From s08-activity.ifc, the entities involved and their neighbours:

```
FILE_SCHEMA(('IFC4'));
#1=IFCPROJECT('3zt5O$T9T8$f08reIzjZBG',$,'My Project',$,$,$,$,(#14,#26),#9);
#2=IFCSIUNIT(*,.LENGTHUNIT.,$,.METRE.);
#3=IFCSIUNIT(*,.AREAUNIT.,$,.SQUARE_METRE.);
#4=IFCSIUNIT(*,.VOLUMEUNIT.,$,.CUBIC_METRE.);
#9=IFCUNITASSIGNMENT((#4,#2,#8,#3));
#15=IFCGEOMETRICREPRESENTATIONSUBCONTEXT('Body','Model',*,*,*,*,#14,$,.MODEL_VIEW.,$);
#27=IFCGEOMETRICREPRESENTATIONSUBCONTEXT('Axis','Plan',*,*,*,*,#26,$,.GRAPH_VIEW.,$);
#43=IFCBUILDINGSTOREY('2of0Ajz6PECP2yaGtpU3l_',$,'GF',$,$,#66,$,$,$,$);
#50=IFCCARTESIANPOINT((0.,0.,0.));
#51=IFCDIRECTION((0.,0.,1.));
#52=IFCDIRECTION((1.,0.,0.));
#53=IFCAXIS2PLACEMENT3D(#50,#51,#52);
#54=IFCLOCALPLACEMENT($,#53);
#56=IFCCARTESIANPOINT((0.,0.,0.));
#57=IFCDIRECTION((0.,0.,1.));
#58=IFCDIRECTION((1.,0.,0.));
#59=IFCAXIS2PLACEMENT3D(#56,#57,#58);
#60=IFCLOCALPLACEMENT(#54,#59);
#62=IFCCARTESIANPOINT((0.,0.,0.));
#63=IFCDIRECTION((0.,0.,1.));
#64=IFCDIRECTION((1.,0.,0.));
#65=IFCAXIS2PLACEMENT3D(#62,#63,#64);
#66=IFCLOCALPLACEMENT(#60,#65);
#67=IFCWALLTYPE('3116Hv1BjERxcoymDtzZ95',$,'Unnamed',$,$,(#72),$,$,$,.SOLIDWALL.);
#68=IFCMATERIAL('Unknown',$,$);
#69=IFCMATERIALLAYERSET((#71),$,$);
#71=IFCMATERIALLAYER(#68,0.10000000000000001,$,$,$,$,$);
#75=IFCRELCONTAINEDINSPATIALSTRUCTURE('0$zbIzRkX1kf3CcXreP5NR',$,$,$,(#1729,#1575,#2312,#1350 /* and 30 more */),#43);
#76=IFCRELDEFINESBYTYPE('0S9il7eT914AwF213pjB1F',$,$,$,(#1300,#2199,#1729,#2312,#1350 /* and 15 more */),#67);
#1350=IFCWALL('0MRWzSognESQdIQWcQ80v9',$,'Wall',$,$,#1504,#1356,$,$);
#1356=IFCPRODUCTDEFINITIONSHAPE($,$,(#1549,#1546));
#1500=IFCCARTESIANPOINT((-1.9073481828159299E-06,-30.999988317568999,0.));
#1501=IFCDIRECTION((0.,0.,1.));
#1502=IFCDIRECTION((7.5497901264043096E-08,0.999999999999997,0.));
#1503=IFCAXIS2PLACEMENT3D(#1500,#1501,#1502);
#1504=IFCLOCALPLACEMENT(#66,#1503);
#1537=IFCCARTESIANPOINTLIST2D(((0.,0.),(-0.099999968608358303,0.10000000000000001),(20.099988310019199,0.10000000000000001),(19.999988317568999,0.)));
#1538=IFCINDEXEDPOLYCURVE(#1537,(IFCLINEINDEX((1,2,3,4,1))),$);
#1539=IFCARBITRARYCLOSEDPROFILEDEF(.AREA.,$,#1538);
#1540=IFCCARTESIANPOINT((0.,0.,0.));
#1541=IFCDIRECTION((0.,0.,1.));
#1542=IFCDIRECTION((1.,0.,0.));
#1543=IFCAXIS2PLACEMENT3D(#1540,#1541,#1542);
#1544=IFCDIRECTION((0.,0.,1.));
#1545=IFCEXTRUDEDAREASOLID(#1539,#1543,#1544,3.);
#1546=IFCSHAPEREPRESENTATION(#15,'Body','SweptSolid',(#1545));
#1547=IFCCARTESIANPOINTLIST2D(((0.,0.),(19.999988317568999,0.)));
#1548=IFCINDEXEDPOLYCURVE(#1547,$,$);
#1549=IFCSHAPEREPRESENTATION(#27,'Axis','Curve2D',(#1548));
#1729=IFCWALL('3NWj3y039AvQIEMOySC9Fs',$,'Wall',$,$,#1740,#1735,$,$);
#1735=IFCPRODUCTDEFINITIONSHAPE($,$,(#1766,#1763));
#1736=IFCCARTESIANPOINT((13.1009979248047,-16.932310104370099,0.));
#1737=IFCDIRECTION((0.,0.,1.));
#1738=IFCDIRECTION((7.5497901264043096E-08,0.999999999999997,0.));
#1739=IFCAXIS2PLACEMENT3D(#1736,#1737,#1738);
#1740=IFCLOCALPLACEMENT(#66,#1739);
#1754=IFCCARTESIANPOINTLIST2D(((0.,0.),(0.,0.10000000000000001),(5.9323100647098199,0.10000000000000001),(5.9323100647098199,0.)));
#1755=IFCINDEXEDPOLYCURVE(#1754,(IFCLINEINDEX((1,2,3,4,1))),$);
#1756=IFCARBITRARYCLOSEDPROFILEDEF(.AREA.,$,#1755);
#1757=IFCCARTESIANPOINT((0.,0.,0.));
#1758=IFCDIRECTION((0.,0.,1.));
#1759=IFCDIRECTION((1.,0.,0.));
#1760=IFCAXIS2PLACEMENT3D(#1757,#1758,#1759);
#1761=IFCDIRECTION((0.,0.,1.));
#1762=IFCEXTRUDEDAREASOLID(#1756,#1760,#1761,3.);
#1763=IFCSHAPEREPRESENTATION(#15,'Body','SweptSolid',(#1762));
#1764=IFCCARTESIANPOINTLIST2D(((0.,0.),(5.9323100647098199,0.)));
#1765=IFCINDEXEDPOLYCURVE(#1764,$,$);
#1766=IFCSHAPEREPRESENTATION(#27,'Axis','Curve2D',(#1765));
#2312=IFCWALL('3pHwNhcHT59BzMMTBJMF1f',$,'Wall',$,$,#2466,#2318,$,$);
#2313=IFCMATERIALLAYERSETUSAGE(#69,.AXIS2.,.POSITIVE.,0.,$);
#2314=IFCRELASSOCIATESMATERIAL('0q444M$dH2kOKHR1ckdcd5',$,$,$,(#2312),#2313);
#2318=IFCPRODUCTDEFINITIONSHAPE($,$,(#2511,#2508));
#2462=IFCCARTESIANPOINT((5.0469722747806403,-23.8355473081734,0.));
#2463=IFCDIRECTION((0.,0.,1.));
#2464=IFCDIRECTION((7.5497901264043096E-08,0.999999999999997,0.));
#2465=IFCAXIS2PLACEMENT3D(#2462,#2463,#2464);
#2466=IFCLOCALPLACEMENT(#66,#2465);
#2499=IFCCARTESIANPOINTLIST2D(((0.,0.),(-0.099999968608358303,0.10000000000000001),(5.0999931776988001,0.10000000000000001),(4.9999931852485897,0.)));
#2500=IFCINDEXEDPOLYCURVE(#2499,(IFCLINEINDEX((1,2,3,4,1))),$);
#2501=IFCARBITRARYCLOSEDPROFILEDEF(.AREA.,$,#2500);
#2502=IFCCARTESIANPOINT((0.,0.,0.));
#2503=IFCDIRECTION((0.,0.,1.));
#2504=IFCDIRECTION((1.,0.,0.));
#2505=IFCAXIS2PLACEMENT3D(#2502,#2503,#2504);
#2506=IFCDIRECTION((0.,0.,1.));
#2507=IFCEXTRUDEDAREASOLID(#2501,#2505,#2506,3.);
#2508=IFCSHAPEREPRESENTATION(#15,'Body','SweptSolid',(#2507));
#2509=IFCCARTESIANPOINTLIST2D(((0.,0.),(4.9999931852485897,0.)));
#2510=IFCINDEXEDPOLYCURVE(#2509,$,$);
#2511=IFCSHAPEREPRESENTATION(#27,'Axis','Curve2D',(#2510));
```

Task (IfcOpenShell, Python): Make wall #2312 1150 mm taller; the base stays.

```python
import ifcopenshell
import ifcopenshell.geom
import ifcopenshell.util.representation
import ifcopenshell.util.shape
import ifcopenshell.util.unit

model = ifcopenshell.open("s08-activity.ifc")
unit_scale = ifcopenshell.util.unit.calculate_unit_scale(model)
settings = ifcopenshell.geom.settings()


def volume(element):
    """Net volume in cubic metres, openings subtracted."""
    shape = ifcopenshell.geom.create_shape(settings, element)
    return ifcopenshell.util.shape.get_volume(shape.geometry)


wall = model.by_guid("3pHwNhcHT59BzMMTBJMF1f")
before = volume(wall)

body = ifcopenshell.util.representation.get_representation(wall, "Model", "Body")
solid = body.Items[0]
old_height = solid.Depth
solid.Depth += 1.15 / unit_scale
after = volume(wall)

print(f"height {old_height:g} -> {solid.Depth:g}, volume {before:.3f} -> {after:.3f} m3")

model.write("s08-activity_updated.ifc")
```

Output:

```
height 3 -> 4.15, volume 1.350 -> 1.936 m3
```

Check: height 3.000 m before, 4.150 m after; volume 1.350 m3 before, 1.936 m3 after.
